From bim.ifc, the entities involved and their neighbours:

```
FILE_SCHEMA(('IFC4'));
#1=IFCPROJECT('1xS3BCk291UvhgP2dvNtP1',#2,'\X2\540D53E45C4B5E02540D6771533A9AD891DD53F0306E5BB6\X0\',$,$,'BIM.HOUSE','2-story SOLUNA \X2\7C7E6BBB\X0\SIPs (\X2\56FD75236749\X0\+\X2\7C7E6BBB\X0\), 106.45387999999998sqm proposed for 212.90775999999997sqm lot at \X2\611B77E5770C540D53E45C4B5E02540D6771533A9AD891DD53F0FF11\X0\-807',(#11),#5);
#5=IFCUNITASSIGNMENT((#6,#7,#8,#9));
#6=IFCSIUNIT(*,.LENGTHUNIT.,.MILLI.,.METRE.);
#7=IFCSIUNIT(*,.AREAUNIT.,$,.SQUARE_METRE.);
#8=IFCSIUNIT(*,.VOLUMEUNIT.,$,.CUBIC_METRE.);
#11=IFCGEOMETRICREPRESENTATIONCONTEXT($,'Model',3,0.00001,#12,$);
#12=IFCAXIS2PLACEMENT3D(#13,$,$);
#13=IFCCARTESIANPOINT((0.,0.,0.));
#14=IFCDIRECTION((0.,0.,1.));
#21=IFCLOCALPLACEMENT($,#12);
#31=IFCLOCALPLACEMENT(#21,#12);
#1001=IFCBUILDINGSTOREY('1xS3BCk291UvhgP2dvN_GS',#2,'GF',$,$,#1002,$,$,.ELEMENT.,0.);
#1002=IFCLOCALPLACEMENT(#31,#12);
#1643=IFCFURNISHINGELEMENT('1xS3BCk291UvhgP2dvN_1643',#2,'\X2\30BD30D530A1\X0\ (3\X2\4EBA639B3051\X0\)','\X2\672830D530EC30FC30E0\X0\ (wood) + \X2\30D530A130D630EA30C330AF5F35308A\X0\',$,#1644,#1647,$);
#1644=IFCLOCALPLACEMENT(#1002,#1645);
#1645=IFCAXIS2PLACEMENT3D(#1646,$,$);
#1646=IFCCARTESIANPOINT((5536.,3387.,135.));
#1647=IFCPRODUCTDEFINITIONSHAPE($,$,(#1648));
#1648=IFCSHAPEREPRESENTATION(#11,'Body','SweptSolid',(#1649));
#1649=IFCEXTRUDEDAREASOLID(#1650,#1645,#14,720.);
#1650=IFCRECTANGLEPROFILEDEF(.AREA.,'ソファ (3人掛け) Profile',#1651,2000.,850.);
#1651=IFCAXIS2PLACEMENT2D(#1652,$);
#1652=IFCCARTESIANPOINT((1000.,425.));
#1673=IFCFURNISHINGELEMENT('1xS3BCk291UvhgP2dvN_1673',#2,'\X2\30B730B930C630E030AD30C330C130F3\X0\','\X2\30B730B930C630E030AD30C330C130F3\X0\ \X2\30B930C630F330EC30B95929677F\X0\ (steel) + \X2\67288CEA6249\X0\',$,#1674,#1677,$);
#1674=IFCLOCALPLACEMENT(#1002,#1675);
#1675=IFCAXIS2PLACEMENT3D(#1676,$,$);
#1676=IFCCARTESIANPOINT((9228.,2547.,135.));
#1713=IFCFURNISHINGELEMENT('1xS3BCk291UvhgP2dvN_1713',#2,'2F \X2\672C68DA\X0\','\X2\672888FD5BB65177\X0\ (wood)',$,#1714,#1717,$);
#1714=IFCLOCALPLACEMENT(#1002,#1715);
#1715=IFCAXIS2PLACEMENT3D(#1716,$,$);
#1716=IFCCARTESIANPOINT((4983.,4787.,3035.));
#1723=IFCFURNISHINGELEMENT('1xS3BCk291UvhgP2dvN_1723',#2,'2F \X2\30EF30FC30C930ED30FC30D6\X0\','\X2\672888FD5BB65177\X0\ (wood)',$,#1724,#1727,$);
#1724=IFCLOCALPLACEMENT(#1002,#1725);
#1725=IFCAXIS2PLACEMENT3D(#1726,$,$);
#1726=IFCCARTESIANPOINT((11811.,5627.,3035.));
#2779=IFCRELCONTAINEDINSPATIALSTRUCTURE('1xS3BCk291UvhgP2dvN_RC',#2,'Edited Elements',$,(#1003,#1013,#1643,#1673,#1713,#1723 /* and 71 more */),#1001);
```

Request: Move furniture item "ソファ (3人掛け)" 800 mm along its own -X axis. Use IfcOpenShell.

```python
import ifcopenshell
import ifcopenshell.api.geometry
import ifcopenshell.util.placement
import ifcopenshell.util.unit

model = ifcopenshell.open("bim.ifc")
unit_scale = ifcopenshell.util.unit.calculate_unit_scale(model)

item = model.by_guid("1xS3BCk291UvhgP2dvN_1643")
matrix = ifcopenshell.util.placement.get_local_placement(item.ObjectPlacement)
matrix[:3, 3] -= matrix[:3, 0] * 0.8 / unit_scale
ifcopenshell.api.geometry.edit_object_placement(model, product=item, matrix=matrix, is_si=False)

print(ifcopenshell.util.placement.get_local_placement(item.ObjectPlacement).round(3) + 0.0)

model.write("bim_v2.ifc")
```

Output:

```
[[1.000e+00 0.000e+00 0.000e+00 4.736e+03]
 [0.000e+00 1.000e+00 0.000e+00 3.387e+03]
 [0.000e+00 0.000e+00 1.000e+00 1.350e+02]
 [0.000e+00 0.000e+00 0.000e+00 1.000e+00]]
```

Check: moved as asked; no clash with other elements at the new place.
